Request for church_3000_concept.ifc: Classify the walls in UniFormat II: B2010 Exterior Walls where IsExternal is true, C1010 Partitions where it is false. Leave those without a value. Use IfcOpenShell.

First a look at what the model holds.

```python
import ifcopenshell
import ifcopenshell.util.element

model = ifcopenshell.open("church_3000_concept.ifc")
print(model.schema)
print("classifications:", [c.Name for c in model.by_type("IfcClassification")])
values = [ifcopenshell.util.element.get_pset(e, "Pset_WallCommon", "IsExternal") for e in model.by_type("IfcWall")]
for value in (True, False, None):
    print("IsExternal", value, values.count(value))
```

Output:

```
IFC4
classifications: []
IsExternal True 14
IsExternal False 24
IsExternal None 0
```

```python
import ifcopenshell
import ifcopenshell.api.classification
import ifcopenshell.util.element

model = ifcopenshell.open("church_3000_concept.ifc")

system = ifcopenshell.api.classification.add_classification(model, classification="UniFormat II")

walls = model.by_type("IfcWall")
external = {e: ifcopenshell.util.element.get_pset(e, "Pset_WallCommon", "IsExternal") for e in walls}
for flag, code, name in ((True, "B2010", "Exterior Walls"), (False, "C1010", "Partitions")):
    products = [e for e in walls if external[e] is flag]
    ifcopenshell.api.classification.add_reference(
        model, products=products, classification=system, identification=code, name=name
    )
    print(code, len(products))

model.write("church_3000_concept_rev.ifc")
```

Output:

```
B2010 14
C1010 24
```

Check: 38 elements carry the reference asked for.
